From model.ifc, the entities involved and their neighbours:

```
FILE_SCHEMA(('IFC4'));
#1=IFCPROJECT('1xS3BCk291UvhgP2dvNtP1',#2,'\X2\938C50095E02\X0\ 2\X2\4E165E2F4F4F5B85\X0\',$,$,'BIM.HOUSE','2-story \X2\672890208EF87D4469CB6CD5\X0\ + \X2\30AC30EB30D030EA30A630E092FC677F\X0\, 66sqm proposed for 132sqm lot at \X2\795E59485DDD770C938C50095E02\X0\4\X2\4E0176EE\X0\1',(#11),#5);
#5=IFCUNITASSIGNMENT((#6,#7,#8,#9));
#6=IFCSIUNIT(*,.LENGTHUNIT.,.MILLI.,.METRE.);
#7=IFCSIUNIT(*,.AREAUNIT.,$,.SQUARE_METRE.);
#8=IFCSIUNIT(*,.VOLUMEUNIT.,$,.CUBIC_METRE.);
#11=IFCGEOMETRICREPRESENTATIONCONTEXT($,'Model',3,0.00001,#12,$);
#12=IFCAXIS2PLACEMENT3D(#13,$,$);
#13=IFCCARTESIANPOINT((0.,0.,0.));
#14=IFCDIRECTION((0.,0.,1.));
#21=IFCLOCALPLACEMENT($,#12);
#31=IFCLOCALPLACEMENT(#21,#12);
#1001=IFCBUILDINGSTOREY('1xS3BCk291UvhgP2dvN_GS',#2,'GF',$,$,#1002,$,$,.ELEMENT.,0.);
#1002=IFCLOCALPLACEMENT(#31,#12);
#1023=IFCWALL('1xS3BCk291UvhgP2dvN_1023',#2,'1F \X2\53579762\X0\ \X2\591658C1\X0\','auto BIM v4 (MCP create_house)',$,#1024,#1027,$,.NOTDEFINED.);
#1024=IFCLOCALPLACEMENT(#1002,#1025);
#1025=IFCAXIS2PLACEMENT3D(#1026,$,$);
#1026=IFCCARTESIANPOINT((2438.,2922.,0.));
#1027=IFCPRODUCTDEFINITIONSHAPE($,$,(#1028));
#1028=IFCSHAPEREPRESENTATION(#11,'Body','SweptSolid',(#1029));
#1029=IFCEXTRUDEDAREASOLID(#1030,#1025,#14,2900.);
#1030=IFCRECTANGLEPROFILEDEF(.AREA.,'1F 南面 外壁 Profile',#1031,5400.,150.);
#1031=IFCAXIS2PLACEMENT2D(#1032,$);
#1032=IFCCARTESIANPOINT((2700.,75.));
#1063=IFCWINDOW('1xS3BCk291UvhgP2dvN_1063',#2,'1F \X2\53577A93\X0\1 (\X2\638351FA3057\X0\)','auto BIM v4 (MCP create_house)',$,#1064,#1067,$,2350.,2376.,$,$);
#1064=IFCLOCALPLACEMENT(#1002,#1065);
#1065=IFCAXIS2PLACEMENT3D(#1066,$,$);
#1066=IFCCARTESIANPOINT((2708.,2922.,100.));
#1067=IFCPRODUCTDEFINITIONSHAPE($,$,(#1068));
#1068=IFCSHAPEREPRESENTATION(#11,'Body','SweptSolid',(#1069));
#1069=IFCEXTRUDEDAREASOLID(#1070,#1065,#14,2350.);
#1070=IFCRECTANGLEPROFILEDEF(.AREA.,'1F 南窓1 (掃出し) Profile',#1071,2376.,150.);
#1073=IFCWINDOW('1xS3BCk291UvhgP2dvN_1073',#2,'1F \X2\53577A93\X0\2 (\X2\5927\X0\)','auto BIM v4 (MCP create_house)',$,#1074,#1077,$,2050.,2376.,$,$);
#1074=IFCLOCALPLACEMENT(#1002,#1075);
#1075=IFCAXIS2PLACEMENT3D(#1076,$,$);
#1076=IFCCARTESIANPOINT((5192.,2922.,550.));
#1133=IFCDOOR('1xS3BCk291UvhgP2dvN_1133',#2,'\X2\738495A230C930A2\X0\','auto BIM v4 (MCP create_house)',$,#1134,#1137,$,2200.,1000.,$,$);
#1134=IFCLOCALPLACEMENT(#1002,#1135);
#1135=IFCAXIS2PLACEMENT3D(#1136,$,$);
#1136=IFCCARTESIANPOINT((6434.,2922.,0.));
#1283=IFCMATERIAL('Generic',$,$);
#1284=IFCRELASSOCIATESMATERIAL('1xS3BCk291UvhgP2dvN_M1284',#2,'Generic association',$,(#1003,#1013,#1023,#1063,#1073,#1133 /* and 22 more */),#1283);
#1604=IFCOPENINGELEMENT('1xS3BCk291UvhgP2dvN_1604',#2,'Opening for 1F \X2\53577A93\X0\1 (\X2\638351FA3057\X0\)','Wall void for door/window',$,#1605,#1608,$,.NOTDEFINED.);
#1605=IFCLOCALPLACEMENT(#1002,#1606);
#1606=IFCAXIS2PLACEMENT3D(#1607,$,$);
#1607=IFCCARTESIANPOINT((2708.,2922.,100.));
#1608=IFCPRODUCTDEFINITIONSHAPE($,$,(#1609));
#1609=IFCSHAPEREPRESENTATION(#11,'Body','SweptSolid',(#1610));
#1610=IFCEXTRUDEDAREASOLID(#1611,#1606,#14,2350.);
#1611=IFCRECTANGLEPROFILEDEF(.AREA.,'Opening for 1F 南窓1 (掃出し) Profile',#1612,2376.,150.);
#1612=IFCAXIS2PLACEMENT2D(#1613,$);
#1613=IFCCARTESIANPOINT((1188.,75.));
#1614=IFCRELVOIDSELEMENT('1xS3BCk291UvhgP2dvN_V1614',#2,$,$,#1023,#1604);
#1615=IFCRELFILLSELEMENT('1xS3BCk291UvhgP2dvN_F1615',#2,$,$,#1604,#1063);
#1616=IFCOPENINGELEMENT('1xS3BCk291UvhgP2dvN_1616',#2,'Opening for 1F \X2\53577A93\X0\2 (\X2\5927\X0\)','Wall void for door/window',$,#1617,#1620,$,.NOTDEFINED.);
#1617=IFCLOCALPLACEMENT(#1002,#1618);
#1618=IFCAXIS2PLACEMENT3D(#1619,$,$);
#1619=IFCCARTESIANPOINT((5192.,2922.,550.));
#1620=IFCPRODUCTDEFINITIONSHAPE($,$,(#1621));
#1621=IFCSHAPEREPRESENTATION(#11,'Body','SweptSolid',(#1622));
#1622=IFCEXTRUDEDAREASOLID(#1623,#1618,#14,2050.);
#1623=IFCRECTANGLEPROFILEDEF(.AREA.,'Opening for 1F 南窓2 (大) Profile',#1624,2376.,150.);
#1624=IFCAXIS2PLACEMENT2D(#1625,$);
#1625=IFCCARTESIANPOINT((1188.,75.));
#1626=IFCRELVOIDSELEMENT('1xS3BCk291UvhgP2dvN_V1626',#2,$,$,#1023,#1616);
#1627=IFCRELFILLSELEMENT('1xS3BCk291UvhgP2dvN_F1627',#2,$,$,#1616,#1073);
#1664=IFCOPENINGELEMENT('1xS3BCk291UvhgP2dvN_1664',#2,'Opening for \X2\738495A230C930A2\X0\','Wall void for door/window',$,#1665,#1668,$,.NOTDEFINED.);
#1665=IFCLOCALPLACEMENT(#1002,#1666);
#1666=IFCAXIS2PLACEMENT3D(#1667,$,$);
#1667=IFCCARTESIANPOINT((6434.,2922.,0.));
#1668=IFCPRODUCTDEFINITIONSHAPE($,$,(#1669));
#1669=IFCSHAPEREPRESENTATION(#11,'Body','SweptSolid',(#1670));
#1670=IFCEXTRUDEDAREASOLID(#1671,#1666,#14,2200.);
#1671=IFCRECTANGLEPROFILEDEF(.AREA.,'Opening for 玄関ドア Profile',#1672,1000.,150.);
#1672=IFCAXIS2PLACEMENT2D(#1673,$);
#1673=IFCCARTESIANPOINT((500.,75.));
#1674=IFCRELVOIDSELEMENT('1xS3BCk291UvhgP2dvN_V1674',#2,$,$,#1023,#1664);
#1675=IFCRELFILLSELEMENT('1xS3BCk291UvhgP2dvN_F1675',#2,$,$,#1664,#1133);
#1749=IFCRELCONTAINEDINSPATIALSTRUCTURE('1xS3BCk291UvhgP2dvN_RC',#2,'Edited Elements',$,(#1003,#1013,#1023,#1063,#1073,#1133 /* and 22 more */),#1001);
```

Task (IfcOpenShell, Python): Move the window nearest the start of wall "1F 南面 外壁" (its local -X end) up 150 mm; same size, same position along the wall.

```python
import numpy as np
import ifcopenshell
import ifcopenshell.api.geometry
import ifcopenshell.util.placement
import ifcopenshell.util.unit

model = ifcopenshell.open("model.ifc")
unit_scale = ifcopenshell.util.unit.calculate_unit_scale(model)

window = model.by_id(1063)
opening = window.FillsVoids[0].RelatingOpeningElement
dz = 0.15 / unit_scale

shift = np.array([0.0, 0.0, dz])
# The window is not placed relative to its opening, so move both.
for product in (opening, window):
    matrix = ifcopenshell.util.placement.get_local_placement(product.ObjectPlacement)
    matrix[:3, 3] += shift
    ifcopenshell.api.geometry.edit_object_placement(model, product=product, matrix=matrix, is_si=False)

print(f"moved by {dz * unit_scale:+.3f} m")

model.write("model_updated.ifc")
```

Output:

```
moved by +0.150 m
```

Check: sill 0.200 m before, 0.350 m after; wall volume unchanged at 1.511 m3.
